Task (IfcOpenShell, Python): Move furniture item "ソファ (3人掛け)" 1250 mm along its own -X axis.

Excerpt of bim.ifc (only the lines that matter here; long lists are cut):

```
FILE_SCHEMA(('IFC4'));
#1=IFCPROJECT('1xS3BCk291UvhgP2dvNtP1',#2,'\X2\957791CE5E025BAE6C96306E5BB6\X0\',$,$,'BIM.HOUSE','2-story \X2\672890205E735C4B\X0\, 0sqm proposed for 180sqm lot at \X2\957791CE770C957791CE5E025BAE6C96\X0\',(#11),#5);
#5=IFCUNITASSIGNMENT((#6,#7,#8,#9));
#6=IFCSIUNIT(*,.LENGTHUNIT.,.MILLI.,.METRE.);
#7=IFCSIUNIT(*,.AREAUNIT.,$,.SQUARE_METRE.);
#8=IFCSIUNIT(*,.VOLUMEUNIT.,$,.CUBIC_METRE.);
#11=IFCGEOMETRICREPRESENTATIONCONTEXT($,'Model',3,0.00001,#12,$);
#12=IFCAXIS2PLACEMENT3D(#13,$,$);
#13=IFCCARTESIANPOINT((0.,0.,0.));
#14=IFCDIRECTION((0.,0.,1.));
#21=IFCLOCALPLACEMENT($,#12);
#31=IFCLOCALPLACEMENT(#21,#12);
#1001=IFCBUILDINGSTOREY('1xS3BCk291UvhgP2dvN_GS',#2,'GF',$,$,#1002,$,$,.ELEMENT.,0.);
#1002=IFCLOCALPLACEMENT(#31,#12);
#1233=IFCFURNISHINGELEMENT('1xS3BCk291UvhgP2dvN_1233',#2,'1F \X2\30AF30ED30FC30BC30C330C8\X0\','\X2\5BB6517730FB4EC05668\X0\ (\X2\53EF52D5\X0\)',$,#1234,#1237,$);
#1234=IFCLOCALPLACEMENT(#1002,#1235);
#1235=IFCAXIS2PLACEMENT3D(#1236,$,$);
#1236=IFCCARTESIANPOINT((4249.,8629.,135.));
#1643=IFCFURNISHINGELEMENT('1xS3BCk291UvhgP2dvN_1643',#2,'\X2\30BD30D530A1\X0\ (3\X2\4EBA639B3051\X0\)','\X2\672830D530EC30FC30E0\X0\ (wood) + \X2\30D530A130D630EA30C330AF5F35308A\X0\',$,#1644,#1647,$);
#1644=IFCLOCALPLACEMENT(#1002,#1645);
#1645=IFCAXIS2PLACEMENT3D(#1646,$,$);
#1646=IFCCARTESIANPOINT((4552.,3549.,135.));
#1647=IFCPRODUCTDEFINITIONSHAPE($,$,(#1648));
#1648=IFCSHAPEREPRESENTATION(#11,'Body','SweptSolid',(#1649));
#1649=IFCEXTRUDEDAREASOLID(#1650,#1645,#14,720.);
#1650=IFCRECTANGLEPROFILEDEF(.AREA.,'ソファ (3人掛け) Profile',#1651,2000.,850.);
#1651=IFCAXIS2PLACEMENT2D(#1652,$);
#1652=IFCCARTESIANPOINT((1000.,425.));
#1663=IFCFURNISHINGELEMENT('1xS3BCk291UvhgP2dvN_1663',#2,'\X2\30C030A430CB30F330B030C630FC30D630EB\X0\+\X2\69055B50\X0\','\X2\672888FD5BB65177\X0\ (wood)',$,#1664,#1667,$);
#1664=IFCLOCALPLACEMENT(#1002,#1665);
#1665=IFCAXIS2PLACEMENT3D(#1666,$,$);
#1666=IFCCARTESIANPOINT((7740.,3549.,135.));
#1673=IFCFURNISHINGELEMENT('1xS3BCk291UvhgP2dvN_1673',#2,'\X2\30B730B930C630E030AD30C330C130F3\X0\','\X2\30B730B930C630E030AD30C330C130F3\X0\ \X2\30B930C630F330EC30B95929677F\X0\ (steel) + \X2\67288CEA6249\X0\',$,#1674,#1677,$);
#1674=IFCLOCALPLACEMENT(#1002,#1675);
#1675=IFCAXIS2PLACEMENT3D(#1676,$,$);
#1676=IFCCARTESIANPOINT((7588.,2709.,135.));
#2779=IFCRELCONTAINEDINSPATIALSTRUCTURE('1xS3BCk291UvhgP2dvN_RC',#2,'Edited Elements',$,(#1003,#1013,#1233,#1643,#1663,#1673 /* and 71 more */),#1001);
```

```python
import ifcopenshell
import ifcopenshell.api.geometry
import ifcopenshell.util.placement

model = ifcopenshell.open("bim.ifc")

item = model.by_guid("1xS3BCk291UvhgP2dvN_1643")
matrix = ifcopenshell.util.placement.get_local_placement(item.ObjectPlacement)
matrix[:3, 3] -= matrix[:3, 0] * 1250.0
ifcopenshell.api.geometry.edit_object_placement(model, product=item, matrix=matrix, is_si=False)

print(ifcopenshell.util.placement.get_local_placement(item.ObjectPlacement).round(3) + 0.0)

model.write("bim_edited.ifc")
```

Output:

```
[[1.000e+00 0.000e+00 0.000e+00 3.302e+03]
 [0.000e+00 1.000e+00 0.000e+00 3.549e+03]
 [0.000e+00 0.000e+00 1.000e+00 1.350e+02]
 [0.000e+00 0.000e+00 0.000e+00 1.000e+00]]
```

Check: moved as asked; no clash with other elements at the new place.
